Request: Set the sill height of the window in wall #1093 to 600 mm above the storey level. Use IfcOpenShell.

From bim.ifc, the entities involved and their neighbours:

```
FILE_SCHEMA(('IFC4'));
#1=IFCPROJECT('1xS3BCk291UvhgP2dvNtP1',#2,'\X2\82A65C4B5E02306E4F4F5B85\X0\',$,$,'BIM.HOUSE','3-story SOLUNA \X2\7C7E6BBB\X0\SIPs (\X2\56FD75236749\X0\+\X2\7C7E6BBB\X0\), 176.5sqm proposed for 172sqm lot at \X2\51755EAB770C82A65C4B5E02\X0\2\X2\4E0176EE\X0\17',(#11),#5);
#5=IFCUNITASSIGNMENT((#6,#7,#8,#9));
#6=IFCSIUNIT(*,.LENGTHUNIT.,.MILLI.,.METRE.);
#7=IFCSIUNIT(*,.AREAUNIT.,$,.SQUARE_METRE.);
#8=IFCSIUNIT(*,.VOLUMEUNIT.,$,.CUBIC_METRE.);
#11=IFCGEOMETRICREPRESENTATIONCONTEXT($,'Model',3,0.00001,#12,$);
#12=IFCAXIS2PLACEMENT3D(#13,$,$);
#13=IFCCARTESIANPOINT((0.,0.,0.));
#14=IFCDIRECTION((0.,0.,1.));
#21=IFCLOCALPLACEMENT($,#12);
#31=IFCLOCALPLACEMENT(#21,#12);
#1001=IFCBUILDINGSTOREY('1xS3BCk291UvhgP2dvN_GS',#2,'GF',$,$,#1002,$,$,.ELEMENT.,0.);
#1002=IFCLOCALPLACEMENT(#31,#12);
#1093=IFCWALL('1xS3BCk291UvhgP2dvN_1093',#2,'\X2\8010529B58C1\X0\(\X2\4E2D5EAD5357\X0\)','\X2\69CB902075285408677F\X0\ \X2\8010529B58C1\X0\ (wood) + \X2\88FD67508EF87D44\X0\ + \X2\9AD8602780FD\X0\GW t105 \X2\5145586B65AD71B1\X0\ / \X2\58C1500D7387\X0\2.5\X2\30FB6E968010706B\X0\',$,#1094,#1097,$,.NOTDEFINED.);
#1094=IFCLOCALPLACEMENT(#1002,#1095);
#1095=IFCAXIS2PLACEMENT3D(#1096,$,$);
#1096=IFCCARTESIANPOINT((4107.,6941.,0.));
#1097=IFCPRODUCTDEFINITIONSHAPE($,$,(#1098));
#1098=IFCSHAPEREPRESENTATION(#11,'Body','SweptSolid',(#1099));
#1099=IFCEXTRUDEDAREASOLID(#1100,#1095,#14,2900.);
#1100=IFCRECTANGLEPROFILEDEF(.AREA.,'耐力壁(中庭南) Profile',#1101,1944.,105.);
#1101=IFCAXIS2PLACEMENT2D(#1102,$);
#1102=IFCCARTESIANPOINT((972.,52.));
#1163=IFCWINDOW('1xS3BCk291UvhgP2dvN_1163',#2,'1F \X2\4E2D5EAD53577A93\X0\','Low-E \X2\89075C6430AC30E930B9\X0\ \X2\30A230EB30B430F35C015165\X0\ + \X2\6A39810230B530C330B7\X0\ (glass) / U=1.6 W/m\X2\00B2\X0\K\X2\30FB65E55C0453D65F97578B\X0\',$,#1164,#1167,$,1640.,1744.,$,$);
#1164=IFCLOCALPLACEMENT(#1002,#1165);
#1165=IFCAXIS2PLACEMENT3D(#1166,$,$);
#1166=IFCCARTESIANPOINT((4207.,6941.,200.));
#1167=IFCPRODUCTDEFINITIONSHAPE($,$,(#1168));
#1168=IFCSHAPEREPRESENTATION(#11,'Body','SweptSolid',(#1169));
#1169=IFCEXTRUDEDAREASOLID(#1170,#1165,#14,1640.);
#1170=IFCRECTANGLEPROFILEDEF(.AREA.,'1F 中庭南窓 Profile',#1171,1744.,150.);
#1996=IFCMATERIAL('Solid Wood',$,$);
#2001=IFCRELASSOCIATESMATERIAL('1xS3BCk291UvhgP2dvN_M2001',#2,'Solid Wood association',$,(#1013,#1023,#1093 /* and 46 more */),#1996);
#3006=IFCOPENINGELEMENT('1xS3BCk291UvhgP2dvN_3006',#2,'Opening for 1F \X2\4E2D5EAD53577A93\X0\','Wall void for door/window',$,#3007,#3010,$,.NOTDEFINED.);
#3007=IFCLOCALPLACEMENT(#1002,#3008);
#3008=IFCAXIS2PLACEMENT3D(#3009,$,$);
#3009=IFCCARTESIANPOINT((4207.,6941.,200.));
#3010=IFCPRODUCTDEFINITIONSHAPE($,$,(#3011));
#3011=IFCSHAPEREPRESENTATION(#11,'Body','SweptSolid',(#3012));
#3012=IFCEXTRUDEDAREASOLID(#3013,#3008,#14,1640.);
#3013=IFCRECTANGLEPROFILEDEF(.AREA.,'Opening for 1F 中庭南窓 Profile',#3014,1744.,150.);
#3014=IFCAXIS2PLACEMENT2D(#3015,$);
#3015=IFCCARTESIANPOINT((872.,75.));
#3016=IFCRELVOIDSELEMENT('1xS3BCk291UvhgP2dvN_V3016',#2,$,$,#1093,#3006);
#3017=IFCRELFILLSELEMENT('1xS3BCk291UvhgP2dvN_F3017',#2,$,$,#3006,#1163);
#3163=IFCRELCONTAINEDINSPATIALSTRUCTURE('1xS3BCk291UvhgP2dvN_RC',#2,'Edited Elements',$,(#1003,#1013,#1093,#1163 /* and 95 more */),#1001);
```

```python
import numpy as np
import ifcopenshell
import ifcopenshell.api.geometry
import ifcopenshell.geom
import ifcopenshell.util.element
import ifcopenshell.util.placement
import ifcopenshell.util.shape
import ifcopenshell.util.unit

model = ifcopenshell.open("bim.ifc")
unit_scale = ifcopenshell.util.unit.calculate_unit_scale(model)

window = model.by_guid("1xS3BCk291UvhgP2dvN_1163")
opening = window.FillsVoids[0].RelatingOpeningElement
storey = ifcopenshell.util.element.get_container(window, ifc_class="IfcBuildingStorey")
level = ifcopenshell.util.placement.get_local_placement(storey.ObjectPlacement)[2, 3]

# The opening's origin need not be at the sill, so measure its lowest point.
shape = ifcopenshell.geom.create_shape(ifcopenshell.geom.settings(), opening)
bottom = ifcopenshell.util.shape.get_shape_bottom_elevation(shape, shape.geometry) / unit_scale
dz = level + 0.6 / unit_scale - bottom

shift = np.array([0.0, 0.0, dz])
# The window is not placed relative to its opening, so move both.
for product in (opening, window):
    matrix = ifcopenshell.util.placement.get_local_placement(product.ObjectPlacement)
    matrix[:3, 3] += shift
    ifcopenshell.api.geometry.edit_object_placement(model, product=product, matrix=matrix, is_si=False)

print(f"moved by {dz * unit_scale:+.3f} m")

model.write("bim_v2.ifc")
```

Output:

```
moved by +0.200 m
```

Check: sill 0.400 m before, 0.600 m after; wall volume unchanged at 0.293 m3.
